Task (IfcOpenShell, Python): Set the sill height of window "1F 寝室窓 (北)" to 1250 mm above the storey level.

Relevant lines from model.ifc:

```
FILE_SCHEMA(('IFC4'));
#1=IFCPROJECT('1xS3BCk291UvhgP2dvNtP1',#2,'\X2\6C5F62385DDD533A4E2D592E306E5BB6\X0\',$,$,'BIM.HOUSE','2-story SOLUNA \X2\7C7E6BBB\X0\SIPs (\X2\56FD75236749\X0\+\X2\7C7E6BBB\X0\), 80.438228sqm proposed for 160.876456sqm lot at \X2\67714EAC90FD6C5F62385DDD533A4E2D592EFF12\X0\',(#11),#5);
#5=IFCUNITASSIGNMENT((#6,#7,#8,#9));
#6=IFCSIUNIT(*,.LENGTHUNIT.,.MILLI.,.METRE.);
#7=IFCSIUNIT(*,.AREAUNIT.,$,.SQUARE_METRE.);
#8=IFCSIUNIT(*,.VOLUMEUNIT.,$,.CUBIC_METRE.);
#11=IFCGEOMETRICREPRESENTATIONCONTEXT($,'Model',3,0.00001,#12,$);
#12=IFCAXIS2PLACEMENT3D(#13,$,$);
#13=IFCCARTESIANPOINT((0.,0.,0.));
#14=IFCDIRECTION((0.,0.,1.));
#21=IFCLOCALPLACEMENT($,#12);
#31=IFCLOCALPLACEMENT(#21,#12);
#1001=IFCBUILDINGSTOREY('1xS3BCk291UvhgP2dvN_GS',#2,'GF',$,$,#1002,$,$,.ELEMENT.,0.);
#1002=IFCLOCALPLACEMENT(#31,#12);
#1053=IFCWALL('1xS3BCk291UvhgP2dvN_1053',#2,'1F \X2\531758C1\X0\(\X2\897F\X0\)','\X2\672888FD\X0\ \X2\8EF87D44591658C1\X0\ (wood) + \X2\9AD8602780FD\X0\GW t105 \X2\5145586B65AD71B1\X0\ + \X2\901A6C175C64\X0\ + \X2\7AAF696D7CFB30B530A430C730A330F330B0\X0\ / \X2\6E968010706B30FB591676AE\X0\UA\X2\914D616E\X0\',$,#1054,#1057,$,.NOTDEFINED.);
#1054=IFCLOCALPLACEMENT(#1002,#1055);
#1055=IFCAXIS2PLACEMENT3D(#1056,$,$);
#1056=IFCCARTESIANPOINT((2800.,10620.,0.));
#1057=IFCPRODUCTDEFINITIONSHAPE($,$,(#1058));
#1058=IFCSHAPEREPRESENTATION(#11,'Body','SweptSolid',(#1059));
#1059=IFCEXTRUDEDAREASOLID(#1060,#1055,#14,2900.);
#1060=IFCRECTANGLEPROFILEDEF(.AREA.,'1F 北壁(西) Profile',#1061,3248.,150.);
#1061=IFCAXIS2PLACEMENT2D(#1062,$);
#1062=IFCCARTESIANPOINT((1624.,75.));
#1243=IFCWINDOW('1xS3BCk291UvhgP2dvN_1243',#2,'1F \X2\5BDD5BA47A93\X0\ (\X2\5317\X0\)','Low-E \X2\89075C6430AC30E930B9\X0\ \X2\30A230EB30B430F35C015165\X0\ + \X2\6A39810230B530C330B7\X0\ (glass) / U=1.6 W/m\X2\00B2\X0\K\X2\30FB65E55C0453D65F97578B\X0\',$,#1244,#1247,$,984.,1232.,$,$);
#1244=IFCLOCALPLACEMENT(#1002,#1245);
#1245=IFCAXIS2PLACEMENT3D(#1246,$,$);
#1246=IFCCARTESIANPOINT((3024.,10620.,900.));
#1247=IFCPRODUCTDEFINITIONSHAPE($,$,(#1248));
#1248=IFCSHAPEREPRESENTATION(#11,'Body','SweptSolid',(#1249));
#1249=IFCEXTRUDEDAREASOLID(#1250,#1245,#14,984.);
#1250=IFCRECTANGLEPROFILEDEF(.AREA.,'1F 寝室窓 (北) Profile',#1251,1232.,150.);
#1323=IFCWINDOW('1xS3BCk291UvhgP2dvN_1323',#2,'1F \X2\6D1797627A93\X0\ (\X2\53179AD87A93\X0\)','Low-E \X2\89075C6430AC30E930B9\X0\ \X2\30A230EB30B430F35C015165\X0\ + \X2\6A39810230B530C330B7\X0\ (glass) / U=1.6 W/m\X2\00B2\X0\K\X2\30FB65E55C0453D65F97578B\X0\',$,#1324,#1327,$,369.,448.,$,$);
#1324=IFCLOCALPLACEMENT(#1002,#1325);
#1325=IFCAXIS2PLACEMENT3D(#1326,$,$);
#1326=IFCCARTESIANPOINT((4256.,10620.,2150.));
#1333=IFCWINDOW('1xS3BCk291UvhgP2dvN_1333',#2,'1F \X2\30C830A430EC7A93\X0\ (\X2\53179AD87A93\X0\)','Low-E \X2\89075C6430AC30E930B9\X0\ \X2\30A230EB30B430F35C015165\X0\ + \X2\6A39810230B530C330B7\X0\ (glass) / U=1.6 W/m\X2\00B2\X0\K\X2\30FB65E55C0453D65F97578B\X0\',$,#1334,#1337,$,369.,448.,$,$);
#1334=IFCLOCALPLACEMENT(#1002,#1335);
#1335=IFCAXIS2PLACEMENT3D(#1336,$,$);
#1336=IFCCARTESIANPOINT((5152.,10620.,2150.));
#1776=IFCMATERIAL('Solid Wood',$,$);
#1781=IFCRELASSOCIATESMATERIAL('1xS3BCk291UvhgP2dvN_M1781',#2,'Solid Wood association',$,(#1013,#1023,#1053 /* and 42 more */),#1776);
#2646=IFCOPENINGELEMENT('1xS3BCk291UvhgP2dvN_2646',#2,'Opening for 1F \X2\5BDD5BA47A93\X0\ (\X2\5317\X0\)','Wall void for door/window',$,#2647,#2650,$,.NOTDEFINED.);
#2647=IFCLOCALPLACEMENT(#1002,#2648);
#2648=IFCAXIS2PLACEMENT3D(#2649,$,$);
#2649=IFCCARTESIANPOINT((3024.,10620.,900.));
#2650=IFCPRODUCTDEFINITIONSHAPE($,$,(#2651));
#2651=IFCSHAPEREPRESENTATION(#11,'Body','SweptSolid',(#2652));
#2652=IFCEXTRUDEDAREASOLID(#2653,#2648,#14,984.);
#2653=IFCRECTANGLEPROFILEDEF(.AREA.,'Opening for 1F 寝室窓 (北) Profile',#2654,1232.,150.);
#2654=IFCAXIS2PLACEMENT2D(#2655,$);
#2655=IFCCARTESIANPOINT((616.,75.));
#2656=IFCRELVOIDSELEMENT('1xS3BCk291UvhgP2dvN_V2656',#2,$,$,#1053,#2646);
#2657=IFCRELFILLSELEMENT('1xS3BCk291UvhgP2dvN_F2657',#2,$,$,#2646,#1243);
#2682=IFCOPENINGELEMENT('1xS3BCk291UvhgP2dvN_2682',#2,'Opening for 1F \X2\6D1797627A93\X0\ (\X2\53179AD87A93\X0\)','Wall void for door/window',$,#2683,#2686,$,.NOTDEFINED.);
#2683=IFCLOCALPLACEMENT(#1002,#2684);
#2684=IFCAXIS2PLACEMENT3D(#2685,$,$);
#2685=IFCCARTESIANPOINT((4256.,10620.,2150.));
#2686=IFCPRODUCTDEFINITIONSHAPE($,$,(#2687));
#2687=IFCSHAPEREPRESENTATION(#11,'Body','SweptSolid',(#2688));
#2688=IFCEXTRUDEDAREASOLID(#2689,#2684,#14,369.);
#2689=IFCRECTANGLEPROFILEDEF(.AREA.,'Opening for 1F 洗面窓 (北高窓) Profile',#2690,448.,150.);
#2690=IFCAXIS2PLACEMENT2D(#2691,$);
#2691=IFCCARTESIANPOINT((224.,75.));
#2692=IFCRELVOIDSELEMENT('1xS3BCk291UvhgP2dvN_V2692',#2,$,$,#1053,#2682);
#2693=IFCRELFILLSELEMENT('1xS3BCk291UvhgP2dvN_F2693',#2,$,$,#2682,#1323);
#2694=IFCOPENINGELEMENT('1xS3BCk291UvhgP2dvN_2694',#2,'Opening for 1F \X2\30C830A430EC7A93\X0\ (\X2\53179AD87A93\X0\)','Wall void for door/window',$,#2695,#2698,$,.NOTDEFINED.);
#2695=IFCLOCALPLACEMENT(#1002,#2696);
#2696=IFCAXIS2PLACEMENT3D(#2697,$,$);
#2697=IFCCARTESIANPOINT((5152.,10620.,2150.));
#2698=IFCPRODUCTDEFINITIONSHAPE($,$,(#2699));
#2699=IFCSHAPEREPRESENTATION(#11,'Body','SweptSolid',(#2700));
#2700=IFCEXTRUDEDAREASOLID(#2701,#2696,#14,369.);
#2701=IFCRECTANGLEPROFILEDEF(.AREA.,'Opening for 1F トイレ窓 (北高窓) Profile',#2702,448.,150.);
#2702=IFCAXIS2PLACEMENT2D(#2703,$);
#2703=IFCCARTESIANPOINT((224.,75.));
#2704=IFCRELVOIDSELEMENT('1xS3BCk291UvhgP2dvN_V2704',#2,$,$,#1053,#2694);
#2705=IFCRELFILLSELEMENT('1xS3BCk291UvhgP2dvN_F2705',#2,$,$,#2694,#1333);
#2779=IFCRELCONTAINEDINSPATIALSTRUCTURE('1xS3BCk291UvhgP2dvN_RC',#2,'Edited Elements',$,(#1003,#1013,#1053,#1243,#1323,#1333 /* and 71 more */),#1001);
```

```python
import numpy as np
import ifcopenshell
import ifcopenshell.api.geometry
import ifcopenshell.geom
import ifcopenshell.util.element
import ifcopenshell.util.placement
import ifcopenshell.util.shape
import ifcopenshell.util.unit

model = ifcopenshell.open("model.ifc")
unit_scale = ifcopenshell.util.unit.calculate_unit_scale(model)

window = model.by_id(1243)
opening = window.FillsVoids[0].RelatingOpeningElement
storey = ifcopenshell.util.element.get_container(window, ifc_class="IfcBuildingStorey")
level = ifcopenshell.util.placement.get_local_placement(storey.ObjectPlacement)[2, 3]

# The opening's origin need not be at the sill, so measure its lowest point.
shape = ifcopenshell.geom.create_shape(ifcopenshell.geom.settings(), opening)
bottom = ifcopenshell.util.shape.get_shape_bottom_elevation(shape, shape.geometry) / unit_scale
dz = level + 1.25 / unit_scale - bottom

shift = np.array([0.0, 0.0, dz])
# The window is not placed relative to its opening, so move both.
for product in (opening, window):
    matrix = ifcopenshell.util.placement.get_local_placement(product.ObjectPlacement)
    matrix[:3, 3] += shift
    ifcopenshell.api.geometry.edit_object_placement(model, product=product, matrix=matrix, is_si=False)

print(f"moved by {dz * unit_scale:+.3f} m")

model.write("model_updated.ifc")
```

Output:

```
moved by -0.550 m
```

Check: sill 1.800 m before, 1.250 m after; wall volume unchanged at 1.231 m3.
